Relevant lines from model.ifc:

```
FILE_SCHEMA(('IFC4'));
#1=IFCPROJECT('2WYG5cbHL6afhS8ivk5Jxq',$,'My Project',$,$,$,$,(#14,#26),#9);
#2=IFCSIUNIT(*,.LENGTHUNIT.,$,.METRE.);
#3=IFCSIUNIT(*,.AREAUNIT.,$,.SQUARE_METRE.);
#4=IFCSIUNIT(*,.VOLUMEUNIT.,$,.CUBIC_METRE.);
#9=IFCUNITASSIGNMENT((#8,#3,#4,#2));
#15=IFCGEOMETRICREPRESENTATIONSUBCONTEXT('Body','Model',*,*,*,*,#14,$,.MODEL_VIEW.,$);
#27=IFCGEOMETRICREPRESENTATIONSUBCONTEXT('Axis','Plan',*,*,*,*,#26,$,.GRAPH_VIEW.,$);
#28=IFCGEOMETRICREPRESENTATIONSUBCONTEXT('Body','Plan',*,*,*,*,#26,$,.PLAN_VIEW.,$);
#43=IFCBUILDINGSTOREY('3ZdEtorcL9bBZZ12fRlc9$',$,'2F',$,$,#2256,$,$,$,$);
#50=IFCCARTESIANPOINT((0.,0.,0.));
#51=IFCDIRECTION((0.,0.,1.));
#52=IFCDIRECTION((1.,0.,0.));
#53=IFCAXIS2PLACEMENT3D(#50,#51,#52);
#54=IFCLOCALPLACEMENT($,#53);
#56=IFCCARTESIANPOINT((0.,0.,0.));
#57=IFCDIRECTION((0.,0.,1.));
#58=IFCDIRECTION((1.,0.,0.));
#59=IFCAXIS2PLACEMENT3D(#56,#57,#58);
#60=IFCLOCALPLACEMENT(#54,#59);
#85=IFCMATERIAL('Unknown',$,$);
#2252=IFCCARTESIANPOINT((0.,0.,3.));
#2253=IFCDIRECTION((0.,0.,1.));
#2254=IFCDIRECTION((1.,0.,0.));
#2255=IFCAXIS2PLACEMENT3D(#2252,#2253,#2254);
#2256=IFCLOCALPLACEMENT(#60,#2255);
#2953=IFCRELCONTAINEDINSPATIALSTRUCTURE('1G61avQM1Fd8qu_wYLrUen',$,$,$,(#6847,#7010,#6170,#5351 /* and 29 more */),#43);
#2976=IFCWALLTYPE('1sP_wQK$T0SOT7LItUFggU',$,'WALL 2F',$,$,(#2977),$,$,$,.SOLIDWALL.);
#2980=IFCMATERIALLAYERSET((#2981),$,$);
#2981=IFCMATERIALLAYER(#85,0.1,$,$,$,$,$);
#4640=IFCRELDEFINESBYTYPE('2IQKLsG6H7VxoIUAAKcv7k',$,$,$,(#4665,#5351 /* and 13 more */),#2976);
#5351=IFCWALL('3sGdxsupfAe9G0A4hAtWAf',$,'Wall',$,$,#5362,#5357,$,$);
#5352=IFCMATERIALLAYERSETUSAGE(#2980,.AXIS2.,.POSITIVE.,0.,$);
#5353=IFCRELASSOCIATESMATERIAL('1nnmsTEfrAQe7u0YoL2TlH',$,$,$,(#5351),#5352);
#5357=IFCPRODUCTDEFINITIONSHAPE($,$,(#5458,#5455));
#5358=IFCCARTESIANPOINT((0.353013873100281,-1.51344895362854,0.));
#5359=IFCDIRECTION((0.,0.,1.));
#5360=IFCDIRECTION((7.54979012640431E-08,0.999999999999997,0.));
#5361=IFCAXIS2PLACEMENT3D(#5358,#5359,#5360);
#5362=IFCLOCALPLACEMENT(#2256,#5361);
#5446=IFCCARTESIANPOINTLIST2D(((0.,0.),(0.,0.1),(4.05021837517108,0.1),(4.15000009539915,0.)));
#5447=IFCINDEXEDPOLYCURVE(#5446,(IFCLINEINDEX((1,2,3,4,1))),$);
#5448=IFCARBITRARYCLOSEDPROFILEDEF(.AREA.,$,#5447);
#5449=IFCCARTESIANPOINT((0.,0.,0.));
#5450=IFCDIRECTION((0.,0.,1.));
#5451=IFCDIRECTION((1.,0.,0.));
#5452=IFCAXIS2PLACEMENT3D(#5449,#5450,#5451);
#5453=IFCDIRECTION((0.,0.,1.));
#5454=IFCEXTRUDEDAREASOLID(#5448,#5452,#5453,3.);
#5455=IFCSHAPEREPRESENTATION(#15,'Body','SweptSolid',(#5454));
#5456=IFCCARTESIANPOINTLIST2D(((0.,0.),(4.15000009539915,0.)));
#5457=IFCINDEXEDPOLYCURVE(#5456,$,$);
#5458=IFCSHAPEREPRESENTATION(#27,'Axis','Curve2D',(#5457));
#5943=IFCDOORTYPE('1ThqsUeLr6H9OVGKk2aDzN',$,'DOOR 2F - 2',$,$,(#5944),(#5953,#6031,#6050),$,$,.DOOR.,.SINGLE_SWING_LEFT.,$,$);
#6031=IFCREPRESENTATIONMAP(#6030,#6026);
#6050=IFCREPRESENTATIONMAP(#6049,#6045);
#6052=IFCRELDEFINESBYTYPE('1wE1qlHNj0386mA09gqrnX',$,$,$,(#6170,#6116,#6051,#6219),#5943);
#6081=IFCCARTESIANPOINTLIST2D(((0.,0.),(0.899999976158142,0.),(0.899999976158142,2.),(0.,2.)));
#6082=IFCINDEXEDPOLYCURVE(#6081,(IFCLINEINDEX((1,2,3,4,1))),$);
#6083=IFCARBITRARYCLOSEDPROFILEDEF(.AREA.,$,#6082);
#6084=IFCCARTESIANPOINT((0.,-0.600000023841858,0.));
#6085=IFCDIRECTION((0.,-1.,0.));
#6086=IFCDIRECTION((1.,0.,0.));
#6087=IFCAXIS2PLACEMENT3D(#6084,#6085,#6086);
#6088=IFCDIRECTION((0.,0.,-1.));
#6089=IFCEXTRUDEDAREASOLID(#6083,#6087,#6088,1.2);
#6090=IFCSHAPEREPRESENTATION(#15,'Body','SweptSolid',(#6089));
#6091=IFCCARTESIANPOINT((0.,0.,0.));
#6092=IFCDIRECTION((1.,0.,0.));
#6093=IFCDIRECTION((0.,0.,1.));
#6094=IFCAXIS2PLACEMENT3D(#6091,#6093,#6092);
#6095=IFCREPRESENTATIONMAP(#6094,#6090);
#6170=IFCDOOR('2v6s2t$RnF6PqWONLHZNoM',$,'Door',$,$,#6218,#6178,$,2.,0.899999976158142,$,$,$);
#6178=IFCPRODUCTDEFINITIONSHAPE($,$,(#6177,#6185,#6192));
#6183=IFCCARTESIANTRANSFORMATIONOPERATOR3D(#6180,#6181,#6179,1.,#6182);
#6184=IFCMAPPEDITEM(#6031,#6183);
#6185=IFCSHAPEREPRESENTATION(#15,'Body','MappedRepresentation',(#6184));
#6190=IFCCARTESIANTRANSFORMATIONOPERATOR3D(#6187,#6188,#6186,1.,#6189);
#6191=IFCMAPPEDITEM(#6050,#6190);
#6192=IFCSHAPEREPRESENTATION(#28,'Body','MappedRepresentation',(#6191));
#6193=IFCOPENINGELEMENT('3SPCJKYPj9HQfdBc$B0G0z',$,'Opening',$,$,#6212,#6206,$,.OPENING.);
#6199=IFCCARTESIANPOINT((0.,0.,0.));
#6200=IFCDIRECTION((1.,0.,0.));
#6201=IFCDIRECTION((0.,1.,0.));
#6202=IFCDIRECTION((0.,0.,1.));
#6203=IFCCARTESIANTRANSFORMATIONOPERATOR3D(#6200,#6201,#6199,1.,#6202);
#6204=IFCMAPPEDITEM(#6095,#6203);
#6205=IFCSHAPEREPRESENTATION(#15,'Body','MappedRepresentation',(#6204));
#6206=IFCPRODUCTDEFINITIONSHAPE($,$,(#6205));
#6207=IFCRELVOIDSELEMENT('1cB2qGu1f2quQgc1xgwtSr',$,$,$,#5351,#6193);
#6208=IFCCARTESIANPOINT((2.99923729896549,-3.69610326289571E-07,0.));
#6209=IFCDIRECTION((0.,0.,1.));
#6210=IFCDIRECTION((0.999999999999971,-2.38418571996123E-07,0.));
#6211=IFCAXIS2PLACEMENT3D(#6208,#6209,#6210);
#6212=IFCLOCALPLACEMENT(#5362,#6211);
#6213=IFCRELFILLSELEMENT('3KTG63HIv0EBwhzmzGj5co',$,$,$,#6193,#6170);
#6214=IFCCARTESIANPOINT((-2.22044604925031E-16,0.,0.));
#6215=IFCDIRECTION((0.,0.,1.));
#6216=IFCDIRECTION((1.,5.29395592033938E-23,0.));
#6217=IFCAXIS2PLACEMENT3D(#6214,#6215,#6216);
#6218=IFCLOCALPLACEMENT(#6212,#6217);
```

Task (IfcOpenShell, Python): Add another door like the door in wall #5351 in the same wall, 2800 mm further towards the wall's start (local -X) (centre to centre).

```python
import ifcopenshell
import ifcopenshell.api.feature
import ifcopenshell.api.geometry
import ifcopenshell.api.root
import ifcopenshell.geom
import ifcopenshell.util.element
import ifcopenshell.util.placement
import ifcopenshell.util.shape
import ifcopenshell.util.unit

model = ifcopenshell.open("model.ifc")
unit_scale = ifcopenshell.util.unit.calculate_unit_scale(model)
settings = ifcopenshell.geom.settings()


def volume(element):
    """Net volume in cubic metres, openings subtracted."""
    shape = ifcopenshell.geom.create_shape(settings, element)
    return ifcopenshell.util.shape.get_volume(shape.geometry)


door = model.by_guid("2v6s2t$RnF6PqWONLHZNoM")
opening = door.FillsVoids[0].RelatingOpeningElement
wall = opening.VoidsElements[0].RelatingBuildingElement
before = volume(wall)
shift = ifcopenshell.util.placement.get_local_placement(wall.ObjectPlacement)[:3, 0] * -2.8 / unit_scale

# copy_class copies the void relationship, type, container and properties, but no geometry.
new_opening = ifcopenshell.api.root.copy_class(model, product=opening)
new_opening.Representation = ifcopenshell.util.element.copy_deep(
    model, opening.Representation, exclude=["IfcGeometricRepresentationContext", "IfcRepresentationMap"]
)
new_door = ifcopenshell.api.root.copy_class(model, product=door)
new_door.Representation = ifcopenshell.util.element.copy_deep(
    model, door.Representation, exclude=["IfcGeometricRepresentationContext", "IfcRepresentationMap"]
)
ifcopenshell.api.feature.add_filling(model, opening=new_opening, element=new_door)

for old, new in ((opening, new_opening), (door, new_door)):
    matrix = ifcopenshell.util.placement.get_local_placement(old.ObjectPlacement)
    matrix[:3, 3] += shift
    ifcopenshell.api.geometry.edit_object_placement(model, product=new, matrix=matrix, is_si=False)

after = volume(wall)

print(f"wall volume {before:.3f} -> {after:.3f} m3")

model.write("model_rev.ifc")
```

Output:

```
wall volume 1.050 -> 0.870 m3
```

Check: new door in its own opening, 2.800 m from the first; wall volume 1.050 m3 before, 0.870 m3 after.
